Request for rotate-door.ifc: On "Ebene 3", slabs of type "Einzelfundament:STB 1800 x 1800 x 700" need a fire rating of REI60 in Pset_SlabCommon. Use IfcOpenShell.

First a look at what the model holds.

```python
import ifcopenshell
import ifcopenshell.util.element

model = ifcopenshell.open("rotate-door.ifc")
print(model.schema)
storey = next(s for s in model.by_type("IfcBuildingStorey") if s.Name == "Ebene 3")
slabs = [e for e in ifcopenshell.util.element.get_decomposition(storey) if e.is_a("IfcSlab")]
seen = {}
for e in slabs:
    element_type = ifcopenshell.util.element.get_type(e)
    key = (element_type.Name if element_type != e and element_type else None, ifcopenshell.util.element.get_pset(e, "Pset_SlabCommon", "FireRating"))
    seen[key] = seen.get(key, 0) + 1
for (name, value), count in sorted(seen.items(), key=str):
    print(count, "x", name, "|", value)
```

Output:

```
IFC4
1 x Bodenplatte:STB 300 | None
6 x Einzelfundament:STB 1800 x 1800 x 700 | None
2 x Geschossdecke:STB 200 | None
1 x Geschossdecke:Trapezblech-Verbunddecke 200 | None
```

```python
import ifcopenshell
import ifcopenshell.api.pset
import ifcopenshell.util.element

model = ifcopenshell.open("rotate-door.ifc")

storey = next(s for s in model.by_type("IfcBuildingStorey") if s.Name == "Ebene 3")
slabs = [e for e in ifcopenshell.util.element.get_decomposition(storey) if e.is_a("IfcSlab")]

count = 0
for e in slabs:
    element_type = ifcopenshell.util.element.get_type(e)
    if element_type in (None, e) or element_type.Name != "Einzelfundament:STB 1800 x 1800 x 700":
        continue
    # add_pset returns the element's existing set when there is one.
    pset = ifcopenshell.api.pset.add_pset(model, product=e, name="Pset_SlabCommon")
    ifcopenshell.api.pset.edit_pset(model, pset=pset, properties={"FireRating": "REI60"})
    count += 1

print(count, "slabs updated")

model.write("rotate-door_updated.ifc")
```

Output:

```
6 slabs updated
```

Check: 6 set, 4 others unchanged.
